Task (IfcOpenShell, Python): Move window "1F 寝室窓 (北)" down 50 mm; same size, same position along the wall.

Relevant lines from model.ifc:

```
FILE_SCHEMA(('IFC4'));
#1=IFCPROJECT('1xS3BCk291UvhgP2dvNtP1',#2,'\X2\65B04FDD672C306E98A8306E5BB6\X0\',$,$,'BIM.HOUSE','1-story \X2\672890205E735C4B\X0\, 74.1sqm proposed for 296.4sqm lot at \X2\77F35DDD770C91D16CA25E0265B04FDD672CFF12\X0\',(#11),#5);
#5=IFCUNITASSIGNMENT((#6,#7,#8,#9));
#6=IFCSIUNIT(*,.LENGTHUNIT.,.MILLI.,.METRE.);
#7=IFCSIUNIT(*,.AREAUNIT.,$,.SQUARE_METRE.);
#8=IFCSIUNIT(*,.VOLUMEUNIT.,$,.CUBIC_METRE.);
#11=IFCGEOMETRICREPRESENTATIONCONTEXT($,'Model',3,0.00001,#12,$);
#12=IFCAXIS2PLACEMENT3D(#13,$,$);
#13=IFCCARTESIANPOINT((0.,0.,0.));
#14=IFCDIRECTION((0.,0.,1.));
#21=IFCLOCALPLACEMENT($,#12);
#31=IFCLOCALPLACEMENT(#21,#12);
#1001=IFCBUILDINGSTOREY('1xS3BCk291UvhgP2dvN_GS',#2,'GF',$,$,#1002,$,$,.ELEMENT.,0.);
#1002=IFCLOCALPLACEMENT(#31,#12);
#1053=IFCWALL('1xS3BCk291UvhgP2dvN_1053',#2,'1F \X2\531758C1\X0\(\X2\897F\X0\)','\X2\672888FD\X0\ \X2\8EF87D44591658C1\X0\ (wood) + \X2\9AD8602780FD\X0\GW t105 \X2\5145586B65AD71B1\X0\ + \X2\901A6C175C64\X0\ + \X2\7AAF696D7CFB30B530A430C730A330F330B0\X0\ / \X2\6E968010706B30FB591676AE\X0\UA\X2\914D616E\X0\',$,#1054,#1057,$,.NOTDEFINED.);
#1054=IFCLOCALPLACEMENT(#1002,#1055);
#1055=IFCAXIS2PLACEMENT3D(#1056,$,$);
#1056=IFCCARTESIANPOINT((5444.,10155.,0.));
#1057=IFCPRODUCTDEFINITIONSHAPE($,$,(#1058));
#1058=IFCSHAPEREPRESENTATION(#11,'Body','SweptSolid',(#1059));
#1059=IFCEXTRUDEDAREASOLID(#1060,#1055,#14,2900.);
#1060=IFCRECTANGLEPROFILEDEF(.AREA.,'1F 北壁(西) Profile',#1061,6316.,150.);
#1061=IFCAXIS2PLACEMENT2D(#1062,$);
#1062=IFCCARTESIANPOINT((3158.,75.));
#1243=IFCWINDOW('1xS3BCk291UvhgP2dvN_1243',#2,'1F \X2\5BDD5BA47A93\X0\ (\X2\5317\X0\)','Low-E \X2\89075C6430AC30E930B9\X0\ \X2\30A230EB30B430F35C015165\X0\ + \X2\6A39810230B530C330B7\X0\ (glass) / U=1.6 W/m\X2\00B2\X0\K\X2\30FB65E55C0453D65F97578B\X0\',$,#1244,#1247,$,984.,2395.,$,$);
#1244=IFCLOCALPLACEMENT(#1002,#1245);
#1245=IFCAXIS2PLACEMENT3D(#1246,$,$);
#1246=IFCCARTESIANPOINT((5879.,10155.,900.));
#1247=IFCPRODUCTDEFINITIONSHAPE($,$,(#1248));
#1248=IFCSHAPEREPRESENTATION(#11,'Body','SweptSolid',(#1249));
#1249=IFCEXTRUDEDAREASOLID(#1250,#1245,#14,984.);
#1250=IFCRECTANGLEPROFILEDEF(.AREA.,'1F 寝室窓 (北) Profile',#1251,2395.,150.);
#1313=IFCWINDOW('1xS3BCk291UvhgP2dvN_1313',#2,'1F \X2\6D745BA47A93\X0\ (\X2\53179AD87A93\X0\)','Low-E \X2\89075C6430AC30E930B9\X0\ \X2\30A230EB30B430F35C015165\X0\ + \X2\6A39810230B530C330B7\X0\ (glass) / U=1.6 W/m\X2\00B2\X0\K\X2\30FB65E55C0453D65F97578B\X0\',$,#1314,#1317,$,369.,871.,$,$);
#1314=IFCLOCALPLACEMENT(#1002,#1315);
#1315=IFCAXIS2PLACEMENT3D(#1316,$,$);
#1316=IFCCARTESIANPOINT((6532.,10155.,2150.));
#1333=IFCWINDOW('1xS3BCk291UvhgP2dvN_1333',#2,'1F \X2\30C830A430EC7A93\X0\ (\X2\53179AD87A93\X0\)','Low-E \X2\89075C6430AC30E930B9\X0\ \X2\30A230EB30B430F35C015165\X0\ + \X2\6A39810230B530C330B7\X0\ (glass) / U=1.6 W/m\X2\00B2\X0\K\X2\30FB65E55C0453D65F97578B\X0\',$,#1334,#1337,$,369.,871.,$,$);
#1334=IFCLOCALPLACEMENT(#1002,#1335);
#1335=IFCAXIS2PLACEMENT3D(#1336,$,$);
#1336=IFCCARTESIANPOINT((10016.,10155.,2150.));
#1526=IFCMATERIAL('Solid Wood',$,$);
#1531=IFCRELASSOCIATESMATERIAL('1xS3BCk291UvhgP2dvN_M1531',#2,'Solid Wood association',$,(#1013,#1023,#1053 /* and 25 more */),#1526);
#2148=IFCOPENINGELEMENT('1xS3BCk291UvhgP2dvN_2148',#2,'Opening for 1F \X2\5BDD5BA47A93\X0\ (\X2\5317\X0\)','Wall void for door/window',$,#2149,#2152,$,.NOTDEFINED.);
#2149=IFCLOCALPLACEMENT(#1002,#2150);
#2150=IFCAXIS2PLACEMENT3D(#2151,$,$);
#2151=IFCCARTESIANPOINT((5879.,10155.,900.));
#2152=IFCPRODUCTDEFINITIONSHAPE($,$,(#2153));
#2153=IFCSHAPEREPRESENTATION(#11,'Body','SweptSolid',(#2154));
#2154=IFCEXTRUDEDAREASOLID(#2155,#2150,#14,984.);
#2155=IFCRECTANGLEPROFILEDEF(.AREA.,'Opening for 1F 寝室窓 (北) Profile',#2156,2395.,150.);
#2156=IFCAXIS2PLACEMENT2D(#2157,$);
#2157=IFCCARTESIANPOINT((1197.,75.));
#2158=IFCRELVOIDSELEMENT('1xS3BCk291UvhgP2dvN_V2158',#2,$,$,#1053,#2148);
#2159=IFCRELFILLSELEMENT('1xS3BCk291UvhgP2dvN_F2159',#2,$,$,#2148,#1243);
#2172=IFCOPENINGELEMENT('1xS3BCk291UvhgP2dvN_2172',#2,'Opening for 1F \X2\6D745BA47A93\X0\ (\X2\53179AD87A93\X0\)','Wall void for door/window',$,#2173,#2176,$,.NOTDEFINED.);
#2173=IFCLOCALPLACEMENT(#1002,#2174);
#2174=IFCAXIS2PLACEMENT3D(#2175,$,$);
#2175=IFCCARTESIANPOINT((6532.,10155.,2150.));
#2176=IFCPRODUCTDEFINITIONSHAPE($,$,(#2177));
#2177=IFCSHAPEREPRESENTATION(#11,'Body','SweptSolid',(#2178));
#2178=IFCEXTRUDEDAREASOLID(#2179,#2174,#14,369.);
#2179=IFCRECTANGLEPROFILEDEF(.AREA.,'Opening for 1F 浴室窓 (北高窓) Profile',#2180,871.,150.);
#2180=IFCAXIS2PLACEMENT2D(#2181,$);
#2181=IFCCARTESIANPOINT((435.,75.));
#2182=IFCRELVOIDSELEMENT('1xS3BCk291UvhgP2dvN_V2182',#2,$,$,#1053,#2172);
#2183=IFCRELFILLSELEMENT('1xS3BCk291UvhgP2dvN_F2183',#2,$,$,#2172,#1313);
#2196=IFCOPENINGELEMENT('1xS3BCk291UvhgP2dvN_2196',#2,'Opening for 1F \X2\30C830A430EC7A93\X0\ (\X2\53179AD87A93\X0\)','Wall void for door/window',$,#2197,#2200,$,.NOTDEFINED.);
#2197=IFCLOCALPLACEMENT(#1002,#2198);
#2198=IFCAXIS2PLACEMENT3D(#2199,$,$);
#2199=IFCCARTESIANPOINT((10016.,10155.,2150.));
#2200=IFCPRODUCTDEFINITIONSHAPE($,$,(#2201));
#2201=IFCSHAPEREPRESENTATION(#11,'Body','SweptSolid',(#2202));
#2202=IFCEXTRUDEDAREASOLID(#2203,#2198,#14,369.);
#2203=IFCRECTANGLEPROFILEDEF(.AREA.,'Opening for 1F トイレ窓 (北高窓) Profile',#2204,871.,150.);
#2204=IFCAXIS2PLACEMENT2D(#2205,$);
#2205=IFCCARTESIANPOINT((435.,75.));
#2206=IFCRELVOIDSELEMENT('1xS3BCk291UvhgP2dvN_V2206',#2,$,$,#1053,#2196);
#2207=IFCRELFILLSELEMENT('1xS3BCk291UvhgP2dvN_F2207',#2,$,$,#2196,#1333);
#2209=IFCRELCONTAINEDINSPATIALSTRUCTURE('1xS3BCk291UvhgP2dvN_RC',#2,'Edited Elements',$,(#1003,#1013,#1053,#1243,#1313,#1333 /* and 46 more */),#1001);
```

```python
import numpy as np
import ifcopenshell
import ifcopenshell.api.geometry
import ifcopenshell.util.placement
import ifcopenshell.util.unit

model = ifcopenshell.open("model.ifc")
unit_scale = ifcopenshell.util.unit.calculate_unit_scale(model)

window = model.by_guid("1xS3BCk291UvhgP2dvN_1243")
opening = window.FillsVoids[0].RelatingOpeningElement
dz = -50.0

shift = np.array([0.0, 0.0, dz])
# The window is not placed relative to its opening, so move both.
for product in (opening, window):
    matrix = ifcopenshell.util.placement.get_local_placement(product.ObjectPlacement)
    matrix[:3, 3] += shift
    ifcopenshell.api.geometry.edit_object_placement(model, product=product, matrix=matrix, is_si=False)

print(f"moved by {dz * unit_scale:+.3f} m")

model.write("model_edited.ifc")
```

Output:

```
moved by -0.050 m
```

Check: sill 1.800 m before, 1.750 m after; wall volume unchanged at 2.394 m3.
